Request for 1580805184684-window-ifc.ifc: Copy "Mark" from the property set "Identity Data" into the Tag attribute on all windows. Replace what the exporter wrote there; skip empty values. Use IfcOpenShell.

First a look at what the model holds.

```python
import ifcopenshell
import ifcopenshell.util.element

model = ifcopenshell.open("1580805184684-window-ifc.ifc")
print(model.schema)
windows = model.by_type("IfcWindow")
print(len(windows), "windows")
for e in windows[:8]:
    source = ifcopenshell.util.element.get_pset(e, "Identity Data", "Mark")
    target = e.Tag
    print(e.id(), repr(source), repr(target), sep=" | ")
```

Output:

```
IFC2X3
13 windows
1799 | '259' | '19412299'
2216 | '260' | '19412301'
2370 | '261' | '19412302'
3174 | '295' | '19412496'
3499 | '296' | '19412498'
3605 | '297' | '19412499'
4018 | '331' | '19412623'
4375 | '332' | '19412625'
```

```python
import ifcopenshell
import ifcopenshell.util.element

model = ifcopenshell.open("1580805184684-window-ifc.ifc")

count = 0
for e in model.by_type("IfcWindow"):
    value = ifcopenshell.util.element.get_pset(e, "Identity Data", "Mark")
    current = e.Tag
    if not value or not value.strip() or current == value:
        continue
    e.Tag = value
    count += 1

print(count, "windows updated")

model.write("1580805184684-window-ifc_edited.ifc")
```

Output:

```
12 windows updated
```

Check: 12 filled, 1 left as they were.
